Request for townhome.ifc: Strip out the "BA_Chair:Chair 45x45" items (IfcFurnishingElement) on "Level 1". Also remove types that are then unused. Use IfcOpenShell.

First a look at what the model holds.

```python
import ifcopenshell
import ifcopenshell.util.element

model = ifcopenshell.open("townhome.ifc")
print(model.schema)
storey = next(s for s in model.by_type("IfcBuildingStorey") if s.Name == "Level 1")
furniture = [e for e in ifcopenshell.util.element.get_decomposition(storey) if e.is_a("IfcFurnishingElement")]
seen = {}
for e in furniture:
    element_type = ifcopenshell.util.element.get_type(e)
    name = element_type.Name if element_type not in (None, e) else None
    seen[name] = seen.get(name, 0) + 1
for name, count in sorted(seen.items(), key=str):
    print(count, "x", name)
```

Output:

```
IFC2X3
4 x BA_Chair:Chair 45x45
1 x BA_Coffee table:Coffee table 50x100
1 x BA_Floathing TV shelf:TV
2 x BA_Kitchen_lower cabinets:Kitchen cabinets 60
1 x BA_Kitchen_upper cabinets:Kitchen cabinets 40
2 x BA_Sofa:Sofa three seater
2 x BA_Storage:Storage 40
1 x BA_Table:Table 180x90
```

```python
import ifcopenshell
import ifcopenshell.api.root
import ifcopenshell.util.element

model = ifcopenshell.open("townhome.ifc")

storey = next(s for s in model.by_type("IfcBuildingStorey") if s.Name == "Level 1")
furniture = [e for e in ifcopenshell.util.element.get_decomposition(storey) if e.is_a("IfcFurnishingElement")]
targets = [e for e in furniture if (t := ifcopenshell.util.element.get_type(e)) not in (None, e) and t.Name == "BA_Chair:Chair 45x45"]
types = {ifcopenshell.util.element.get_type(e) for e in targets} - {None, *targets}

for e in targets:
    ifcopenshell.api.root.remove_product(model, product=e)
print(len(targets), "removed")

unused = [t for t in types if not ifcopenshell.util.element.get_types(t)]
for t in unused:
    ifcopenshell.api.root.remove_product(model, product=t)
print(len(unused), "unused types removed")

model.write("townhome_v2.ifc")
```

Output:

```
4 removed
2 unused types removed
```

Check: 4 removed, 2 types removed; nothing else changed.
